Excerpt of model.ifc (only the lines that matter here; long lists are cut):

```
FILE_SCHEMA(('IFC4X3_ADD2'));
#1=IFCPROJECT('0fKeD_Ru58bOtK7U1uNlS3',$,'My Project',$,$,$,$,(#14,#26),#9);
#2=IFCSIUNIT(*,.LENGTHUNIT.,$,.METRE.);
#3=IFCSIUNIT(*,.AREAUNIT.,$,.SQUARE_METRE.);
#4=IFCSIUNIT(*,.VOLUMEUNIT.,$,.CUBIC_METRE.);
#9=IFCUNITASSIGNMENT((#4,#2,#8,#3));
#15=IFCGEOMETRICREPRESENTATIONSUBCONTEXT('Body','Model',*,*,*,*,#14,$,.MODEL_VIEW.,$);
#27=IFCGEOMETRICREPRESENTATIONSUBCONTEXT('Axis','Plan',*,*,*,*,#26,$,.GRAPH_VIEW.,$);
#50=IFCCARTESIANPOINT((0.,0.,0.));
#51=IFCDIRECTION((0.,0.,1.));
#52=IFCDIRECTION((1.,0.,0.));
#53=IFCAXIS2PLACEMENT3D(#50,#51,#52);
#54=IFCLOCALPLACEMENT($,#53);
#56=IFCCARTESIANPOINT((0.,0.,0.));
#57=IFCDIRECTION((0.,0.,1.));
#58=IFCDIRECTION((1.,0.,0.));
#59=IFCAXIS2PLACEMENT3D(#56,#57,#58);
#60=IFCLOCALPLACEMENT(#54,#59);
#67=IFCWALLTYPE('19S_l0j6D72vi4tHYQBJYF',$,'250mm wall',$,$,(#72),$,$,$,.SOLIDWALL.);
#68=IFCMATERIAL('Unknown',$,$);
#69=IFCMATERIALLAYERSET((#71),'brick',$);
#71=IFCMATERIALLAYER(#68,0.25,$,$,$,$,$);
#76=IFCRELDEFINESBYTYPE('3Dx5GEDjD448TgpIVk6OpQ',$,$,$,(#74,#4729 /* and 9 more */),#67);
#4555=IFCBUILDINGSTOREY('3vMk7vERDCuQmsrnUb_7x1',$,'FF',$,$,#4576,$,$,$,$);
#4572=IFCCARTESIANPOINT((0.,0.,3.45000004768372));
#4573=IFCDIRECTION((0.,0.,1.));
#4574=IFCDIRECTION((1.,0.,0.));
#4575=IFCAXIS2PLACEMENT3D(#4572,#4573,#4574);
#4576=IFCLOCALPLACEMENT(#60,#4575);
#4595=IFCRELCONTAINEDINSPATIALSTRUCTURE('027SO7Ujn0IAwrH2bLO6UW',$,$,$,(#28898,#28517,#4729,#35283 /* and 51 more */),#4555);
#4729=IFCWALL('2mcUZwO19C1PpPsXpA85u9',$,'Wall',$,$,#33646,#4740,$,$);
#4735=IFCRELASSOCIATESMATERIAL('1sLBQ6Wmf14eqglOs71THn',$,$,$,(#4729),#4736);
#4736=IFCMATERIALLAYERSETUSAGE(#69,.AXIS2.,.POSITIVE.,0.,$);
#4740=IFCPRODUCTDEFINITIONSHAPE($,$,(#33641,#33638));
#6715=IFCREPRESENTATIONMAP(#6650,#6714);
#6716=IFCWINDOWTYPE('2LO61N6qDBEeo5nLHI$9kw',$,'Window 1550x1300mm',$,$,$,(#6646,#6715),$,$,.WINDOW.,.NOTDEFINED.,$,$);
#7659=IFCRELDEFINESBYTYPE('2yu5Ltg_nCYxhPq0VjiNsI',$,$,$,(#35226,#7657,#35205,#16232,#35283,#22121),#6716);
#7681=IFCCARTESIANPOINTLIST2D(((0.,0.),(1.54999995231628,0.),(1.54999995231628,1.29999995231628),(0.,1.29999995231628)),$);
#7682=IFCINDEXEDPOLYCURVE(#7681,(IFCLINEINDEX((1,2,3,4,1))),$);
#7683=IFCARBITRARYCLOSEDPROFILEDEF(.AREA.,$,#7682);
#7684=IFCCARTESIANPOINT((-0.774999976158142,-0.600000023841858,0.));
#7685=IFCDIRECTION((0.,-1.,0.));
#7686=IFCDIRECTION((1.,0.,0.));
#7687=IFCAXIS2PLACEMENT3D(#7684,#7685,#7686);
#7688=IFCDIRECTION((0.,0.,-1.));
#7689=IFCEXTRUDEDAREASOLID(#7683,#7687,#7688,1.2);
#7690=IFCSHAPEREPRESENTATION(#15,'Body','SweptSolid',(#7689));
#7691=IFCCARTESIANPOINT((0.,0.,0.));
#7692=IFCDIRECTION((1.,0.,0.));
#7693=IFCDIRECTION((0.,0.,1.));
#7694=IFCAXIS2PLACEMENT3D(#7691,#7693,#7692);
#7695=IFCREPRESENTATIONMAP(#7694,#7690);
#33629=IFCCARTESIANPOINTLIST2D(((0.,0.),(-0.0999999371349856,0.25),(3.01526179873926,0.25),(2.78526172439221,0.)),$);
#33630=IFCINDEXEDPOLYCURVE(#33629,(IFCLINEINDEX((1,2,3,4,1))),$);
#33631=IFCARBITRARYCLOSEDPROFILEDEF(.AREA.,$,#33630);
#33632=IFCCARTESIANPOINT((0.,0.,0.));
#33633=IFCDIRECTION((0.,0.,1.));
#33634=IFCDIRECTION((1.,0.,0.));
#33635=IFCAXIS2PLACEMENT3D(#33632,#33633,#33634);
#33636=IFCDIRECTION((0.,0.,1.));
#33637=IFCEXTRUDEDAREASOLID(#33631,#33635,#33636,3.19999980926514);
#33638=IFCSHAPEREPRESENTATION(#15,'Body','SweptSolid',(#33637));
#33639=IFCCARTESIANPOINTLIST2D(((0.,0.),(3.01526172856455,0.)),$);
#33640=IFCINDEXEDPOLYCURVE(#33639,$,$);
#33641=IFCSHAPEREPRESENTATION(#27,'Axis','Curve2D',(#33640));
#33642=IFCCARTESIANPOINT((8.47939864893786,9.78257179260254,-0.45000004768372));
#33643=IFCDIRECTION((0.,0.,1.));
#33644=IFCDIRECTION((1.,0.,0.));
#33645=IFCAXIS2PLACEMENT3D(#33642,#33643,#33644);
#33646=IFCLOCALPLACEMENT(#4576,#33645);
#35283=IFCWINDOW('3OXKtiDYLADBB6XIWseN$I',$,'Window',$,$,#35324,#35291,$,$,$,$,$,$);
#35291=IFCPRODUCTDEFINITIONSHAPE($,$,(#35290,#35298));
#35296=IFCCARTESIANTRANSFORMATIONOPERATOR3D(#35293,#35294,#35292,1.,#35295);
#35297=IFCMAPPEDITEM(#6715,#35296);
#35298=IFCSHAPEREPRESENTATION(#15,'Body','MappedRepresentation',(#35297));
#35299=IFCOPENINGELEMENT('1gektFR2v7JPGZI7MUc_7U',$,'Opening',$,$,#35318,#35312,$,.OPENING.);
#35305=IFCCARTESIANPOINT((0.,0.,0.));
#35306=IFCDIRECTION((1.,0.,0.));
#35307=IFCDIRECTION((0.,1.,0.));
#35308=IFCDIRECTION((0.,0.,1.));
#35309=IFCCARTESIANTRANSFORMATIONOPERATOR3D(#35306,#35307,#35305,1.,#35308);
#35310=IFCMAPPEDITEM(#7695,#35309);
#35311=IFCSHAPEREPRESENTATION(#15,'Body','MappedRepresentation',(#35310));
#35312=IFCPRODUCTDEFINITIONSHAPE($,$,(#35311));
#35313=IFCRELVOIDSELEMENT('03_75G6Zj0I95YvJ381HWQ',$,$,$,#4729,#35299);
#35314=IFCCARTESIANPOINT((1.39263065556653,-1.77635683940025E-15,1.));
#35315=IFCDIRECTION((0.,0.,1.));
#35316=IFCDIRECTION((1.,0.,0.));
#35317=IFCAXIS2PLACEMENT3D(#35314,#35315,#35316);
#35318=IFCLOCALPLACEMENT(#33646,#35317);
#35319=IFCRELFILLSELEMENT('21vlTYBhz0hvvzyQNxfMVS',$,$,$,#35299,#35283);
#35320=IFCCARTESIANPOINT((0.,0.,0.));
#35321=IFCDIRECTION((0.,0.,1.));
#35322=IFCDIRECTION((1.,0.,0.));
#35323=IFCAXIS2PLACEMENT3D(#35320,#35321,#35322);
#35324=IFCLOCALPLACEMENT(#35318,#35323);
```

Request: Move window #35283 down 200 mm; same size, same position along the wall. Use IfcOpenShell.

```python
import numpy as np
import ifcopenshell
import ifcopenshell.api.geometry
import ifcopenshell.util.placement
import ifcopenshell.util.unit

model = ifcopenshell.open("model.ifc")
unit_scale = ifcopenshell.util.unit.calculate_unit_scale(model)

window = model.by_guid("3OXKtiDYLADBB6XIWseN$I")
opening = window.FillsVoids[0].RelatingOpeningElement
dz = -0.2 / unit_scale

shift = np.array([0.0, 0.0, dz])
# The window is placed relative to its opening, so it follows when the opening moves.
matrix = ifcopenshell.util.placement.get_local_placement(opening.ObjectPlacement)
matrix[:3, 3] += shift
ifcopenshell.api.geometry.edit_object_placement(
    model, product=opening, matrix=matrix, is_si=False, should_transform_children=True
)

print(f"moved by {dz * unit_scale:+.3f} m")

model.write("model_rev.ifc")
```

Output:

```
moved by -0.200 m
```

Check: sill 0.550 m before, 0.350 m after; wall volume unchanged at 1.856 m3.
